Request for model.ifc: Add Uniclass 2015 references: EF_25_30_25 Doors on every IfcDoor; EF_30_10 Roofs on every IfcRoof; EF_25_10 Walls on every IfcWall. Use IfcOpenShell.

First a look at what the model holds.

```python
import ifcopenshell

model = ifcopenshell.open("model.ifc")
print(model.schema)
print("classifications:", [c.Name for c in model.by_type("IfcClassification")])
for ifc_class in ("IfcDoor", "IfcRoof", "IfcStair", "IfcWall", "IfcWindow"):
    print(ifc_class, len(model.by_type(ifc_class)))
```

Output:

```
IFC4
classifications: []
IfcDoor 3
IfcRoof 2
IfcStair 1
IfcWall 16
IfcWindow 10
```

```python
import ifcopenshell
import ifcopenshell.api.classification

model = ifcopenshell.open("model.ifc")

system = ifcopenshell.api.classification.add_classification(model, classification="Uniclass 2015")

codes = {
    "IfcDoor": ("EF_25_30_25", "Doors"),
    "IfcRoof": ("EF_30_10", "Roofs"),
    "IfcWall": ("EF_25_10", "Walls"),
}
for ifc_class, (code, name) in codes.items():
    products = model.by_type(ifc_class)
    ifcopenshell.api.classification.add_reference(
        model, products=products, classification=system, identification=code, name=name
    )
    print(code, len(products))

model.write("model-out.ifc")
```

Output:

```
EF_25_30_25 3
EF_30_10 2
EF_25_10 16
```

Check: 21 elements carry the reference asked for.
